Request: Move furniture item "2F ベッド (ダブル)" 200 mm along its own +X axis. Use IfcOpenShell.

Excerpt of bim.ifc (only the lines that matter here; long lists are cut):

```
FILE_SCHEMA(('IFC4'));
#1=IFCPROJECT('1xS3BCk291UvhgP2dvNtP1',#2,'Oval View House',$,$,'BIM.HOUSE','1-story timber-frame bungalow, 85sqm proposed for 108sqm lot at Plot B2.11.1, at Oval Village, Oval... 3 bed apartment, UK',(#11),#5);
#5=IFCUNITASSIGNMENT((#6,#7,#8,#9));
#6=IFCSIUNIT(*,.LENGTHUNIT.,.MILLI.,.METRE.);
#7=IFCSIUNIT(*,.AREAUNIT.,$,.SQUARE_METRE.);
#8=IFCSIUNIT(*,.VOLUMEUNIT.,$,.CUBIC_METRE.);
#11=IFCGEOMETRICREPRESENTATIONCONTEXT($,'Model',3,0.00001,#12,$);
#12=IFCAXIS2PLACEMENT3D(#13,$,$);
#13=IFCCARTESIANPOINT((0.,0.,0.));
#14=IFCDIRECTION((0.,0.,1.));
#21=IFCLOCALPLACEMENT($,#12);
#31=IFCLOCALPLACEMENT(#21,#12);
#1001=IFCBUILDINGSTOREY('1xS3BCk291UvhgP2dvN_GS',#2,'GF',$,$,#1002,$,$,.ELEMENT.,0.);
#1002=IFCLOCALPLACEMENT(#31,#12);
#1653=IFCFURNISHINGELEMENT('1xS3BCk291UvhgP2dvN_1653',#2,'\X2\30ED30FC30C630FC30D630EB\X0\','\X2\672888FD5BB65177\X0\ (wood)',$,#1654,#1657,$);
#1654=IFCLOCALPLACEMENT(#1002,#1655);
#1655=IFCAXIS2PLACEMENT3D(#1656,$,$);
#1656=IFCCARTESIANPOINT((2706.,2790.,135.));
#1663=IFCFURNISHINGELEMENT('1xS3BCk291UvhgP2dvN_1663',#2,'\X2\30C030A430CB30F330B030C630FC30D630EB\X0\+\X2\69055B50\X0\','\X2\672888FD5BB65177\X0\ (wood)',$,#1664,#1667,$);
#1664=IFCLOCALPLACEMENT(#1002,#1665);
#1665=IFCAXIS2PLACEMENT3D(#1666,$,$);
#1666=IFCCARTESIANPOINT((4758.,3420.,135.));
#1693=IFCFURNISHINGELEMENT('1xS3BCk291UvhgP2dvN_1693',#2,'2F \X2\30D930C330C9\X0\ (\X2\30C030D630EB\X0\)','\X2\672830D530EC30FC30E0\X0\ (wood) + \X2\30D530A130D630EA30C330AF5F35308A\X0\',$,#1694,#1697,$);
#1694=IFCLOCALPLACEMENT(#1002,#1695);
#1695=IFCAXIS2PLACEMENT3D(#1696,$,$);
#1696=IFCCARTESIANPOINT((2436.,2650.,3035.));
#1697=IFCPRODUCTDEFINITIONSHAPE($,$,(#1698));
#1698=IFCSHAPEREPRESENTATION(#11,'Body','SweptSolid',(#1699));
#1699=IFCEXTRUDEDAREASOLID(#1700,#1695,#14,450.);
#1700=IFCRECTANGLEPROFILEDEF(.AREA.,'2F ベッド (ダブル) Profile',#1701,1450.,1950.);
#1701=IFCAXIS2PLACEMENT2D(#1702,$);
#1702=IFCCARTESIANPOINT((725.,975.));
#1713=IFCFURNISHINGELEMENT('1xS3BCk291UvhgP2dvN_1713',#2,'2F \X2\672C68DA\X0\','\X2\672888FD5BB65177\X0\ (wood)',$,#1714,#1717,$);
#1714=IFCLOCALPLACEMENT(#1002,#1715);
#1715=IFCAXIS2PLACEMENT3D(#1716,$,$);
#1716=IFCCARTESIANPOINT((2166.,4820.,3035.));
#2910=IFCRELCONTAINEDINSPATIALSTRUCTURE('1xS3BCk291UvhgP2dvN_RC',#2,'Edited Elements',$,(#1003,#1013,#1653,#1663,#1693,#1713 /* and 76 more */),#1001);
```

```python
import ifcopenshell
import ifcopenshell.api.geometry
import ifcopenshell.util.placement

model = ifcopenshell.open("bim.ifc")

item = model.by_guid("1xS3BCk291UvhgP2dvN_1693")
matrix = ifcopenshell.util.placement.get_local_placement(item.ObjectPlacement)
matrix[:3, 3] += matrix[:3, 0] * 200.0
ifcopenshell.api.geometry.edit_object_placement(model, product=item, matrix=matrix, is_si=False)

print(ifcopenshell.util.placement.get_local_placement(item.ObjectPlacement).round(3) + 0.0)

model.write("bim_updated.ifc")
```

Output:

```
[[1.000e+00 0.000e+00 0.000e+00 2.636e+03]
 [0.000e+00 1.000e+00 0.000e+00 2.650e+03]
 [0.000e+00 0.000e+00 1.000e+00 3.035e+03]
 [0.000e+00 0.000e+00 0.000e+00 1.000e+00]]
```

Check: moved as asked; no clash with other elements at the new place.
